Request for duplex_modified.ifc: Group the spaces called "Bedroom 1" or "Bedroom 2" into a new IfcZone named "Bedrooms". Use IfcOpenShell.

First a look at what the model holds.

```python
import ifcopenshell

model = ifcopenshell.open("duplex_modified.ifc")
print(model.schema)
seen = {}
for space in model.by_type("IfcSpace"):
    seen[space.LongName] = seen.get(space.LongName, 0) + 1
for name, count in sorted(seen.items(), key=str):
    print(count, "x", name)
print("zones:", [z.Name for z in model.by_type("IfcZone")][:20])
```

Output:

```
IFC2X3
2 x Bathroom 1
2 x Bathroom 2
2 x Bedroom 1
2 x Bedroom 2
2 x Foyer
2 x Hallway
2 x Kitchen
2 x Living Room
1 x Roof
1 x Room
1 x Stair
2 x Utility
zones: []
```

```python
import ifcopenshell
import ifcopenshell.api.group
import ifcopenshell.api.root

model = ifcopenshell.open("duplex_modified.ifc")

names = {"Bedroom 1", "Bedroom 2"}
spaces = [s for s in model.by_type("IfcSpace") if s.LongName in names]

zone = ifcopenshell.api.root.create_entity(model, ifc_class="IfcZone", name="Bedrooms")
ifcopenshell.api.group.assign_group(model, products=spaces, group=zone)
print(len(spaces), "spaces in", zone.Name)

model.write("duplex_modified_edited.ifc")
```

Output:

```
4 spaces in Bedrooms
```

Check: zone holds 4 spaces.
